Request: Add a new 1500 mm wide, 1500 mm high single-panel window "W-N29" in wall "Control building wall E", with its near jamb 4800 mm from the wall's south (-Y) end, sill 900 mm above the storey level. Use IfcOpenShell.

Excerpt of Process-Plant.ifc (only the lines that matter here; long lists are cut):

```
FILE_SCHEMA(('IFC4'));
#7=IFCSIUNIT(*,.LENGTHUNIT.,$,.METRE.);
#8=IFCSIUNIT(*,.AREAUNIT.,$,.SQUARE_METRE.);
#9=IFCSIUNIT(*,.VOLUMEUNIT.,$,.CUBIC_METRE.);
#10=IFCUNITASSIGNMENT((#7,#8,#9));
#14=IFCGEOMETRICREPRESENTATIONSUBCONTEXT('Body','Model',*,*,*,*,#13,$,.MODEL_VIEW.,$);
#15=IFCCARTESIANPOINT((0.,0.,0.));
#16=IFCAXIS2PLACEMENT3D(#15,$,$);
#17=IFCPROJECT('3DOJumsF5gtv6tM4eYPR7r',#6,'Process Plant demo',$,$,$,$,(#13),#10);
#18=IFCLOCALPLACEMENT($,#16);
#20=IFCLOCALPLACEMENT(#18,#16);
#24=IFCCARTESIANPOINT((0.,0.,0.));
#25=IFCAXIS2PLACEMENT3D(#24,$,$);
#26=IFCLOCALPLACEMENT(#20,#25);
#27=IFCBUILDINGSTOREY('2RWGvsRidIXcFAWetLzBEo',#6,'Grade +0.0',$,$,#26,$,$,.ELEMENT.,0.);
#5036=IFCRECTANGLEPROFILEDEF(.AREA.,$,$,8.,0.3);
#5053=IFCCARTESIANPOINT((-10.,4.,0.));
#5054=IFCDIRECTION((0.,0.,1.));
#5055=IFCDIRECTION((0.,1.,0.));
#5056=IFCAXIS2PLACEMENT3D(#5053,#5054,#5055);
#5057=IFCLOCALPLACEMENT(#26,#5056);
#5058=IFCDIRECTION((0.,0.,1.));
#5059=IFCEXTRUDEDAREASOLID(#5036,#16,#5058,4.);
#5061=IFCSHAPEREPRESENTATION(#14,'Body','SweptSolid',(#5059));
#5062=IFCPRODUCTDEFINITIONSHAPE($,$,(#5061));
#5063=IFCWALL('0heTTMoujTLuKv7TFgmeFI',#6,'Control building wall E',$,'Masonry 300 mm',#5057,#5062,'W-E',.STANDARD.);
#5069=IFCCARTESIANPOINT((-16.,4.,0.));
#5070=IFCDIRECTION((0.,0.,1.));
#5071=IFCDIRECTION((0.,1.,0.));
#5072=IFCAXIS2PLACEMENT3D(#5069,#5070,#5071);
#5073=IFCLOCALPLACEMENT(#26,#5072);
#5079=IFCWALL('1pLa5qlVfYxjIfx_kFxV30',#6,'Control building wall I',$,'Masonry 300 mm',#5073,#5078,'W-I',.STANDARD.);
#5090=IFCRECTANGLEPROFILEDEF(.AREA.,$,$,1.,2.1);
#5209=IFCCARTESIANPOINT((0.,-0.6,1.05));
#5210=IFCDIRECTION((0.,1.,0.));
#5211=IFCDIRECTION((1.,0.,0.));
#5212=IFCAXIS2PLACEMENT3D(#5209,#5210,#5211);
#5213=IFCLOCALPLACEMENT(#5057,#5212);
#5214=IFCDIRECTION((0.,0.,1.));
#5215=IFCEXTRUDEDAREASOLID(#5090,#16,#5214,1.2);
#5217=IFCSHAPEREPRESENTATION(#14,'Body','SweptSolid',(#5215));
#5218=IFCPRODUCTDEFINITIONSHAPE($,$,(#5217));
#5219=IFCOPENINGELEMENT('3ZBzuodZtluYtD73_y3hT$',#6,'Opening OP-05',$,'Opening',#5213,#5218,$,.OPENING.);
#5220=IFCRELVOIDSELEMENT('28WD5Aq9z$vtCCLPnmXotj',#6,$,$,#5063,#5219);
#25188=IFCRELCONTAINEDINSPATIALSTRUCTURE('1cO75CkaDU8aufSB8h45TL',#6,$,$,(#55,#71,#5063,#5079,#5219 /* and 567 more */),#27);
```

```python
import numpy as np
import ifcopenshell
import ifcopenshell.api.feature
import ifcopenshell.api.geometry
import ifcopenshell.api.root
import ifcopenshell.api.spatial
import ifcopenshell.geom
import ifcopenshell.util.element
import ifcopenshell.util.placement
import ifcopenshell.util.representation
import ifcopenshell.util.shape
import ifcopenshell.util.unit

model = ifcopenshell.open("Process-Plant.ifc")
unit_scale = ifcopenshell.util.unit.calculate_unit_scale(model)
settings = ifcopenshell.geom.settings()


def volume(element):
    """Net volume in cubic metres, openings subtracted."""
    shape = ifcopenshell.geom.create_shape(settings, element)
    return ifcopenshell.util.shape.get_volume(shape.geometry)


wall = model.by_id(5063)
storey = ifcopenshell.util.element.get_container(wall, ifc_class="IfcBuildingStorey")
context = ifcopenshell.util.representation.get_context(model, "Model", "Body", "MODEL_VIEW")
before = volume(wall)

width, height, from_end, sill = 1.5, 1.5, 4.8, 0.9  # metres

# The wall runs along its own X axis, and the end named is its -X end.
wall_shape = ifcopenshell.geom.create_shape(settings, wall)
x, y, z = ifcopenshell.util.shape.get_vertices(wall_shape.geometry).T
start = x.min() + from_end
face, thickness = float(y.min()), float(y.max() - y.min())
wall_matrix = ifcopenshell.util.placement.get_local_placement(wall.ObjectPlacement)
level = ifcopenshell.util.placement.get_local_placement(storey.ObjectPlacement)[2, 3]


def in_wall(x, y):
    """Placement at x, y metres in the wall's axes, at sill height."""
    matrix = wall_matrix.copy()
    matrix[:, 3] = wall_matrix @ np.array([x / unit_scale, y / unit_scale, 0.0, 1.0])
    matrix[2, 3] = level + sill / unit_scale
    return matrix


# Opening: a box that overshoots both wall faces by 50 mm.
opening = ifcopenshell.api.root.create_entity(model, ifc_class="IfcOpeningElement", predefined_type="OPENING")
box = ifcopenshell.api.geometry.add_wall_representation(
    model, context=context, length=width, height=height, thickness=thickness + 0.1
)
ifcopenshell.api.geometry.assign_representation(model, product=opening, representation=box)
ifcopenshell.api.geometry.edit_object_placement(model, product=opening, matrix=in_wall(start, face - 0.05), is_si=False)
ifcopenshell.api.feature.add_feature(model, feature=opening, element=wall)

window = ifcopenshell.api.root.create_entity(model, ifc_class="IfcWindow", name="W-N29", predefined_type="WINDOW")
window.OverallWidth, window.OverallHeight = width / unit_scale, height / unit_scale
window.PartitioningType = "SINGLE_PANEL"
body = ifcopenshell.api.geometry.add_window_representation(
    model,
    context=context,
    overall_width=window.OverallWidth,
    overall_height=window.OverallHeight,
    partition_type="SINGLE_PANEL",
)
ifcopenshell.api.geometry.assign_representation(model, product=window, representation=body)
ifcopenshell.api.spatial.assign_container(model, products=[window], relating_structure=storey)
ifcopenshell.api.feature.add_filling(model, opening=opening, element=window)

# Centre the window in the wall's thickness.
ifcopenshell.api.geometry.edit_object_placement(model, product=window, matrix=in_wall(start, face), is_si=False)
window_shape = ifcopenshell.geom.create_shape(settings, window)
depth = ifcopenshell.util.shape.get_vertices(window_shape.geometry)[:, 1]
offset = face + thickness / 2 - (depth.min() + depth.max()) / 2
ifcopenshell.api.geometry.edit_object_placement(model, product=window, matrix=in_wall(start, offset), is_si=False)

after = volume(wall)

print(f"wall volume {before:.3f} -> {after:.3f} m3")

model.write("Process-Plant_edited.ifc")
```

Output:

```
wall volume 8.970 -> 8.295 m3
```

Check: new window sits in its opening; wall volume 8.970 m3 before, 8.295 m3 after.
